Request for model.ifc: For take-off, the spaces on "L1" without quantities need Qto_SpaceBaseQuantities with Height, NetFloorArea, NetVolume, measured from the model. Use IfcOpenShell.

First a look at what the model holds.

```python
import ifcopenshell
import ifcopenshell.util.element
import ifcopenshell.util.unit

model = ifcopenshell.open("model.ifc")
print(model.schema)
for unit_type in ("LENGTHUNIT", "AREAUNIT", "VOLUMEUNIT"):
    print(unit_type, ifcopenshell.util.unit.calculate_unit_scale(model, unit_type))
storey = next(s for s in model.by_type("IfcBuildingStorey") if s.Name == "L1")
spaces = [e for e in ifcopenshell.util.element.get_decomposition(storey) if e.is_a("IfcSpace")]
for e in sorted(spaces, key=lambda e: e.id()):
    print(e.id(), e.is_a(), e.Name, list(ifcopenshell.util.element.get_psets(e, qtos_only=True)), sep=" | ")
```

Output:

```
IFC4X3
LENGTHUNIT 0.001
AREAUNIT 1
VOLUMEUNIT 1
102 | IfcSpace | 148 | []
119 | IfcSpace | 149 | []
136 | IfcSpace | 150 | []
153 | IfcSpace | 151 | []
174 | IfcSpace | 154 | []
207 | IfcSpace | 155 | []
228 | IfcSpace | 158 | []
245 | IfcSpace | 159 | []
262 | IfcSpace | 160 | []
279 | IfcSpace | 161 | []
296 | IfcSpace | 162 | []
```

```python
import ifcopenshell
import ifcopenshell.api.pset
import ifcopenshell.geom
import ifcopenshell.util.element
import ifcopenshell.util.shape
import ifcopenshell.util.unit

model = ifcopenshell.open("model.ifc")
unit_scale = ifcopenshell.util.unit.calculate_unit_scale(model)
area_scale = ifcopenshell.util.unit.calculate_unit_scale(model, "AREAUNIT")
volume_scale = ifcopenshell.util.unit.calculate_unit_scale(model, "VOLUMEUNIT")
settings = ifcopenshell.geom.settings()

storey = next(s for s in model.by_type("IfcBuildingStorey") if s.Name == "L1")
spaces = [e for e in ifcopenshell.util.element.get_decomposition(storey) if e.is_a("IfcSpace")]

for e in sorted(spaces, key=lambda e: e.id()):
    if ifcopenshell.util.element.get_psets(e, qtos_only=True, should_inherit=False):
        continue
    # Geometry comes back in metres, in the element's own axes.
    shape = ifcopenshell.geom.create_shape(settings, e)
    values = {
        "Height": ifcopenshell.util.shape.get_z(shape.geometry) / unit_scale,
        "NetFloorArea": ifcopenshell.util.shape.get_footprint_area(shape.geometry) / area_scale,
        "NetVolume": ifcopenshell.util.shape.get_volume(shape.geometry) / volume_scale,
    }
    qto = ifcopenshell.api.pset.add_qto(model, product=e, name="Qto_SpaceBaseQuantities")
    ifcopenshell.api.pset.edit_qto(model, qto=qto, properties=values)
    print(e.id(), {k: round(v, 3) for k, v in values.items()})

model.write("model_edited.ifc")
```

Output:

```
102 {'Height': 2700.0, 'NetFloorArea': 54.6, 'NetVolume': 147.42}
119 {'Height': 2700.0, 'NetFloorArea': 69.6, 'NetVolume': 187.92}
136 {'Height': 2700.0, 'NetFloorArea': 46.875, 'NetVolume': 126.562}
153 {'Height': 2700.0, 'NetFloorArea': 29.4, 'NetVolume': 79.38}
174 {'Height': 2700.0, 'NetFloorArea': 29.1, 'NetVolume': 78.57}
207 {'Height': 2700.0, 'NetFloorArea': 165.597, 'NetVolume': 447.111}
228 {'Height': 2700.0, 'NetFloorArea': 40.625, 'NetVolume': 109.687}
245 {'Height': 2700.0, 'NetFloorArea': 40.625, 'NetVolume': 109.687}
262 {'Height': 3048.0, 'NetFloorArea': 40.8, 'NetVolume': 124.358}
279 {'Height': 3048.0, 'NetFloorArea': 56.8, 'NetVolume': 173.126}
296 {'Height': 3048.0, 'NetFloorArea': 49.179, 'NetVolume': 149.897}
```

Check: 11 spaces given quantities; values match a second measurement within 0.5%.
